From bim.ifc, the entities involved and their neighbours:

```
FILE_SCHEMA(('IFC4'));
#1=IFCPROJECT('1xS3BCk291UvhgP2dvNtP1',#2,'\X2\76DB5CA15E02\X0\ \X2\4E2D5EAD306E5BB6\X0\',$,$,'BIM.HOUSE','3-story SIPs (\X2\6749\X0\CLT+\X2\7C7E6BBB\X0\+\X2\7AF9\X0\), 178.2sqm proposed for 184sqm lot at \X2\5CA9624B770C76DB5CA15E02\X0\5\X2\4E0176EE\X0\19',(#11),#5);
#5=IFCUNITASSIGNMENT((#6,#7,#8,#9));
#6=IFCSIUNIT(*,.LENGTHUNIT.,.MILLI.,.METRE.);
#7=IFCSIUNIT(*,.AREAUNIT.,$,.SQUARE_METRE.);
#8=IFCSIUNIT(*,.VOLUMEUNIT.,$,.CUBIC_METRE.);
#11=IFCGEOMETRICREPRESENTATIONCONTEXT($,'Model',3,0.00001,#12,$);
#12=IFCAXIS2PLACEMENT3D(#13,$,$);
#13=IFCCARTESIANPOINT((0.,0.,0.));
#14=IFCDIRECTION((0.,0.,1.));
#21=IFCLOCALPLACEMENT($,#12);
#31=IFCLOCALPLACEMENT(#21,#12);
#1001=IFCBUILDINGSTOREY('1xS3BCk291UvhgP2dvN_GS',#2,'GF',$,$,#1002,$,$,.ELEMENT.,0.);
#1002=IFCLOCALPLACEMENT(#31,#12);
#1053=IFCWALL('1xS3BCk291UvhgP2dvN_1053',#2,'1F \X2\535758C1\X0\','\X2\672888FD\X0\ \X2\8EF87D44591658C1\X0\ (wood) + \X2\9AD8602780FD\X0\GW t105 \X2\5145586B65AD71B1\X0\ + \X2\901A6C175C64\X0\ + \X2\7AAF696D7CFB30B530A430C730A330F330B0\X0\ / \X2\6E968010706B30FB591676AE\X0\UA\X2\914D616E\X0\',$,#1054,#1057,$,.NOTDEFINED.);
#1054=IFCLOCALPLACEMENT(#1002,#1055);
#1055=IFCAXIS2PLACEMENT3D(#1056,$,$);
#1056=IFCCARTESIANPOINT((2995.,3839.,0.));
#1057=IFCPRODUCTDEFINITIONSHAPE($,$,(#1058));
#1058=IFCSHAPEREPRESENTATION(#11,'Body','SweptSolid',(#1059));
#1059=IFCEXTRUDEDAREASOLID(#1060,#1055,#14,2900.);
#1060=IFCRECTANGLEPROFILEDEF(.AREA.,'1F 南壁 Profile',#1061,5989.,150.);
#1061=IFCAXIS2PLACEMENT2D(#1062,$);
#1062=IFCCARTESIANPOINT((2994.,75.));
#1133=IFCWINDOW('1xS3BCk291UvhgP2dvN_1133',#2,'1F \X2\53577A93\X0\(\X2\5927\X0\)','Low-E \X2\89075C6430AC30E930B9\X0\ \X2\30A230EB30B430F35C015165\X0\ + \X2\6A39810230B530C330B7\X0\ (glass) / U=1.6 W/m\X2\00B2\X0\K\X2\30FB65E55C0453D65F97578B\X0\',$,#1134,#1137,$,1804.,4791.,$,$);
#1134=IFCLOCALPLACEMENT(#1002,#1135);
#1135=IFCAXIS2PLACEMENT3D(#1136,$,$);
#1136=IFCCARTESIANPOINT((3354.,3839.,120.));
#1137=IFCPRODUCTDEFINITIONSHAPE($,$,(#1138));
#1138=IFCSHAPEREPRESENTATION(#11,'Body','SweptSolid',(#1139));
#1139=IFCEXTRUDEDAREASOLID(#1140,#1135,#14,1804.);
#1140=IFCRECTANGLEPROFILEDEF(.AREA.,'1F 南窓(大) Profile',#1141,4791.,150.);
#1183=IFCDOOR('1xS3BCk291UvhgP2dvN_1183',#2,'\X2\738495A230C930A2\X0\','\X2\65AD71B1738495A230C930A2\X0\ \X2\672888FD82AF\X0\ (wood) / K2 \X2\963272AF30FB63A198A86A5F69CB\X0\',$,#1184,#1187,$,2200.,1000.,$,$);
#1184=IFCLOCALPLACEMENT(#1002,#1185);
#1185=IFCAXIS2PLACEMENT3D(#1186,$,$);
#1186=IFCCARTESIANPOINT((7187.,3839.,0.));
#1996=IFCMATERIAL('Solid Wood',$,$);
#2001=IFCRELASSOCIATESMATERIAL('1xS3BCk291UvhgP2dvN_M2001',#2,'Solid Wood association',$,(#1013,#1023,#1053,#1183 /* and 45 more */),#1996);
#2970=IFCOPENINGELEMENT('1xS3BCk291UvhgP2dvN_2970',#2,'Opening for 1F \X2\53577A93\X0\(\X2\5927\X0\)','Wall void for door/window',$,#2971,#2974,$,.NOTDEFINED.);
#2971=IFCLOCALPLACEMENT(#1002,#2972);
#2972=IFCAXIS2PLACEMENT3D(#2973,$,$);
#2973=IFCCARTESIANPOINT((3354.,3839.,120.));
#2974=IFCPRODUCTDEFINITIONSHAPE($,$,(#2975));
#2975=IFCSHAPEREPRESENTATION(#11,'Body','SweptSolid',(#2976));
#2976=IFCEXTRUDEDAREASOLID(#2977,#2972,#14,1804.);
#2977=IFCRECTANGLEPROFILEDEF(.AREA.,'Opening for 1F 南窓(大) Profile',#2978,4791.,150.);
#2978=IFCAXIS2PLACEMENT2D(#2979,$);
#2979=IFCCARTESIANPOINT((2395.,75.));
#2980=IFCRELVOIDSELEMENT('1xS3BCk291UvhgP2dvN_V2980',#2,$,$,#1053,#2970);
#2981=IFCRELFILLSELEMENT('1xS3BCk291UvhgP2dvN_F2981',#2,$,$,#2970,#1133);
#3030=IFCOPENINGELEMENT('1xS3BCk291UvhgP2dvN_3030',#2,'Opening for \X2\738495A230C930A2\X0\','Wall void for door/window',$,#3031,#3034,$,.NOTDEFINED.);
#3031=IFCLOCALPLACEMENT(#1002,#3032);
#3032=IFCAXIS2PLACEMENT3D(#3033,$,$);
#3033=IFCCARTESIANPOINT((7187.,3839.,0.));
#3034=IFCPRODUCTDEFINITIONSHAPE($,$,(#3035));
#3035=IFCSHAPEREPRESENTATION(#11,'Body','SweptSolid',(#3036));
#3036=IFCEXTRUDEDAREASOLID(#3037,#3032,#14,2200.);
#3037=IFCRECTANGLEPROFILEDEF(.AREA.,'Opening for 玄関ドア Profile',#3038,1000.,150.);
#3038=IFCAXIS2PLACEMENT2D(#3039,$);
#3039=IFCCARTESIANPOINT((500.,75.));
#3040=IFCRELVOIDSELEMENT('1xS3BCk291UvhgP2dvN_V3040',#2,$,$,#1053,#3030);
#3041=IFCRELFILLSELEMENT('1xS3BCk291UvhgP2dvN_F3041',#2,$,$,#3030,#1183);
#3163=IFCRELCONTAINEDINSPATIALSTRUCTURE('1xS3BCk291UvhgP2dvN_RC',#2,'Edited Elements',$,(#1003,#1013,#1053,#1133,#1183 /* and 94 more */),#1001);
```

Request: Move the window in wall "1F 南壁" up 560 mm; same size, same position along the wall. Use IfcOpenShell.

```python
import numpy as np
import ifcopenshell
import ifcopenshell.api.geometry
import ifcopenshell.util.placement
import ifcopenshell.util.unit

model = ifcopenshell.open("bim.ifc")
unit_scale = ifcopenshell.util.unit.calculate_unit_scale(model)

window = model.by_guid("1xS3BCk291UvhgP2dvN_1133")
opening = window.FillsVoids[0].RelatingOpeningElement
dz = 560.0

shift = np.array([0.0, 0.0, dz])
# The window is not placed relative to its opening, so move both.
for product in (opening, window):
    matrix = ifcopenshell.util.placement.get_local_placement(product.ObjectPlacement)
    matrix[:3, 3] += shift
    ifcopenshell.api.geometry.edit_object_placement(model, product=product, matrix=matrix, is_si=False)

print(f"moved by {dz * unit_scale:+.3f} m")

model.write("bim_updated.ifc")
```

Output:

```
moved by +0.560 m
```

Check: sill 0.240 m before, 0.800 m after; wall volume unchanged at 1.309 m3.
